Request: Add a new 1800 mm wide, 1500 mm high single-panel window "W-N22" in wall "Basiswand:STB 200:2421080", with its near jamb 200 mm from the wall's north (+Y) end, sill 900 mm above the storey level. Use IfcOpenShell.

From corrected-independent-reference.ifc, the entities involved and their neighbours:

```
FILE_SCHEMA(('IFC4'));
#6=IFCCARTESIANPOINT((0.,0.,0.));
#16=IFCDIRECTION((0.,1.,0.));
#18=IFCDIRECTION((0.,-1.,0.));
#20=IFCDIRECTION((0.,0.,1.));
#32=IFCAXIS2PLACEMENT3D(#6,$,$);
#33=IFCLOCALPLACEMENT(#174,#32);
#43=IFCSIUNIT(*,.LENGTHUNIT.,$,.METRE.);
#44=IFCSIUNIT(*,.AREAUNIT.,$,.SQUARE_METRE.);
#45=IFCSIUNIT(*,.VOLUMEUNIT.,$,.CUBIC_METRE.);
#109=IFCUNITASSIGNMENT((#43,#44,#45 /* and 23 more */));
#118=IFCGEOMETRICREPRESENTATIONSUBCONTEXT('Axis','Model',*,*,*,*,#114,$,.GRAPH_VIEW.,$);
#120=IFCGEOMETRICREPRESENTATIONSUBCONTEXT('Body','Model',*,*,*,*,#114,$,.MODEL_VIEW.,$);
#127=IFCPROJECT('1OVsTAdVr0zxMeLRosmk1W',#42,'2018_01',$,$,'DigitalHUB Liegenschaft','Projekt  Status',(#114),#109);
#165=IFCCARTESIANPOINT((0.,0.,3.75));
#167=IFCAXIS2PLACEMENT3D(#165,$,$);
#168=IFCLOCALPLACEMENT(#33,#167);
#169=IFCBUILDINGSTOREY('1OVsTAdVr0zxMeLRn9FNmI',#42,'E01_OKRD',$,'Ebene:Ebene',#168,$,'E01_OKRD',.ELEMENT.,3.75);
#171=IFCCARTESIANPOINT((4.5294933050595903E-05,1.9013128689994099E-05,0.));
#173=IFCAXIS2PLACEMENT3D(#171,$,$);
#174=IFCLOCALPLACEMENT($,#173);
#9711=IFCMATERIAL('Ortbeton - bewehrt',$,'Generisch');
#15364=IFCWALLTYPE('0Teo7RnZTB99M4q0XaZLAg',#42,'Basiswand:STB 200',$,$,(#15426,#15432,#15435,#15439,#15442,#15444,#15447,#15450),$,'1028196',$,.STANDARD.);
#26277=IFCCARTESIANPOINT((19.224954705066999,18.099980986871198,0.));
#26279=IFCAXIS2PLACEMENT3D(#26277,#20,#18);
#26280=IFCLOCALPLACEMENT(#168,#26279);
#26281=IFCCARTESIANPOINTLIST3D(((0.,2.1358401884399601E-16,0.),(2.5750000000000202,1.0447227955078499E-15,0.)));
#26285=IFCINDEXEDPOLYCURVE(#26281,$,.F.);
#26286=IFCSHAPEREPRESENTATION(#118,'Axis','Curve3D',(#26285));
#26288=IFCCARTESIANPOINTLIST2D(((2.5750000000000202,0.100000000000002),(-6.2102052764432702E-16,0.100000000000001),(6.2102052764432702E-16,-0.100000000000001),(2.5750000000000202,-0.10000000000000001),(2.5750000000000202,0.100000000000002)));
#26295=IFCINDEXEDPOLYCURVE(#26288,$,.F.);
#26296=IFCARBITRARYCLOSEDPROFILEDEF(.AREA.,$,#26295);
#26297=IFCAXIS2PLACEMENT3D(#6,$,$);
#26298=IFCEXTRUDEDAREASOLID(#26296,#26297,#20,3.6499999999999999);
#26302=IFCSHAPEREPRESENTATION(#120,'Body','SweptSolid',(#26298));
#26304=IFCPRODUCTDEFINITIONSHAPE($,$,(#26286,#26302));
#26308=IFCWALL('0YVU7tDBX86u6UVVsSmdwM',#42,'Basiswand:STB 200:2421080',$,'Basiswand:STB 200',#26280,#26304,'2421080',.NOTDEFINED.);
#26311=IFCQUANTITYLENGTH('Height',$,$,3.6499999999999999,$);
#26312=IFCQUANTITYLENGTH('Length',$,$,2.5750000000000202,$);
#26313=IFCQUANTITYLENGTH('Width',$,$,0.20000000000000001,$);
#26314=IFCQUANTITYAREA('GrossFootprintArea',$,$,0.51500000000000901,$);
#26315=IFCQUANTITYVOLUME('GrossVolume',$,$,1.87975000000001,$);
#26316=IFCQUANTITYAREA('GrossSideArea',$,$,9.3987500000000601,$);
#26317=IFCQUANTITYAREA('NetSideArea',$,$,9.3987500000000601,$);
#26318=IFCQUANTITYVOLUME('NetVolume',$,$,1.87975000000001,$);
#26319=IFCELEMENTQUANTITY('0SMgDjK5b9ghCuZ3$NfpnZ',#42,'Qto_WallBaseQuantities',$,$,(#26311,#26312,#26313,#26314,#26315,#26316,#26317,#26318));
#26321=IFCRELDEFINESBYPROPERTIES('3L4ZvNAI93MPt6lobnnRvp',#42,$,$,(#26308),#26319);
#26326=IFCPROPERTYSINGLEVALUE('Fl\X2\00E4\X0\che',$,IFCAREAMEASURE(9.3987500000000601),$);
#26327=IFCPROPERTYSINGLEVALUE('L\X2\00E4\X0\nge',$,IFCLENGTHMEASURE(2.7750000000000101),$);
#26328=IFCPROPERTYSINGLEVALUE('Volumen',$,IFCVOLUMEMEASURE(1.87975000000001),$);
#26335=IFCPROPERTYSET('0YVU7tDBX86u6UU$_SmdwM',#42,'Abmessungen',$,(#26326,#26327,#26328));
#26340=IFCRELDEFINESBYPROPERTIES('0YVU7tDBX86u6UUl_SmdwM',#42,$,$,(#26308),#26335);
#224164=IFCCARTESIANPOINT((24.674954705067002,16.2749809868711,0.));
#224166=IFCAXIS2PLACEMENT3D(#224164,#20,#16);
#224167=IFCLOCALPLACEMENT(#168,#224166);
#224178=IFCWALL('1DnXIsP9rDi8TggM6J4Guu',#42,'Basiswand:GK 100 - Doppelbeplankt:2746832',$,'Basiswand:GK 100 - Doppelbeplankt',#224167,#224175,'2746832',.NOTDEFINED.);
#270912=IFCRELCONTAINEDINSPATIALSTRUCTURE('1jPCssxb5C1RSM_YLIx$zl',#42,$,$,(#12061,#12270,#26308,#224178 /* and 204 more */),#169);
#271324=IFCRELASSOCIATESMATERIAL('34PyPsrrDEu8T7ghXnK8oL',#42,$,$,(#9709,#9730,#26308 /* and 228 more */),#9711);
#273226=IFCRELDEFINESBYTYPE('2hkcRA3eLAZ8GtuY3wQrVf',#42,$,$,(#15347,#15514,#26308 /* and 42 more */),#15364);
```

```python
import numpy as np
import ifcopenshell
import ifcopenshell.api.feature
import ifcopenshell.api.geometry
import ifcopenshell.api.pset
import ifcopenshell.api.root
import ifcopenshell.api.spatial
import ifcopenshell.geom
import ifcopenshell.util.element
import ifcopenshell.util.placement
import ifcopenshell.util.representation
import ifcopenshell.util.shape
import ifcopenshell.util.unit

model = ifcopenshell.open("corrected-independent-reference.ifc")
unit_scale = ifcopenshell.util.unit.calculate_unit_scale(model)
area_scale = ifcopenshell.util.unit.calculate_unit_scale(model, "AREAUNIT")
volume_scale = ifcopenshell.util.unit.calculate_unit_scale(model, "VOLUMEUNIT")
settings = ifcopenshell.geom.settings()


def volume(element):
    """Net volume in cubic metres, openings subtracted."""
    shape = ifcopenshell.geom.create_shape(settings, element)
    return ifcopenshell.util.shape.get_volume(shape.geometry)


wall = model.by_guid("0YVU7tDBX86u6UVVsSmdwM")
storey = ifcopenshell.util.element.get_container(wall, ifc_class="IfcBuildingStorey")
context = ifcopenshell.util.representation.get_context(model, "Model", "Body", "MODEL_VIEW")
before = volume(wall)

width, height, from_end, sill = 1.8, 1.5, 0.2, 0.9  # metres

# The wall runs along its own X axis, and the end named is its -X end.
wall_shape = ifcopenshell.geom.create_shape(settings, wall)
x, y, z = ifcopenshell.util.shape.get_vertices(wall_shape.geometry).T
start = x.min() + from_end
face, thickness = float(y.min()), float(y.max() - y.min())
wall_matrix = ifcopenshell.util.placement.get_local_placement(wall.ObjectPlacement)
level = ifcopenshell.util.placement.get_local_placement(storey.ObjectPlacement)[2, 3]


def in_wall(x, y):
    """Placement at x, y metres in the wall's axes, at sill height."""
    matrix = wall_matrix.copy()
    matrix[:, 3] = wall_matrix @ np.array([x / unit_scale, y / unit_scale, 0.0, 1.0])
    matrix[2, 3] = level + sill / unit_scale
    return matrix


# Opening: a box that overshoots both wall faces by 50 mm.
opening = ifcopenshell.api.root.create_entity(model, ifc_class="IfcOpeningElement", predefined_type="OPENING")
box = ifcopenshell.api.geometry.add_wall_representation(
    model, context=context, length=width, height=height, thickness=thickness + 0.1
)
ifcopenshell.api.geometry.assign_representation(model, product=opening, representation=box)
ifcopenshell.api.geometry.edit_object_placement(model, product=opening, matrix=in_wall(start, face - 0.05), is_si=False)
ifcopenshell.api.feature.add_feature(model, feature=opening, element=wall)

window = ifcopenshell.api.root.create_entity(model, ifc_class="IfcWindow", name="W-N22", predefined_type="WINDOW")
window.OverallWidth, window.OverallHeight = width / unit_scale, height / unit_scale
window.PartitioningType = "SINGLE_PANEL"
body = ifcopenshell.api.geometry.add_window_representation(
    model,
    context=context,
    overall_width=window.OverallWidth,
    overall_height=window.OverallHeight,
    partition_type="SINGLE_PANEL",
)
ifcopenshell.api.geometry.assign_representation(model, product=window, representation=body)
ifcopenshell.api.spatial.assign_container(model, products=[window], relating_structure=storey)
ifcopenshell.api.feature.add_filling(model, opening=opening, element=window)

# Centre the window in the wall's thickness.
ifcopenshell.api.geometry.edit_object_placement(model, product=window, matrix=in_wall(start, face), is_si=False)
window_shape = ifcopenshell.geom.create_shape(settings, window)
depth = ifcopenshell.util.shape.get_vertices(window_shape.geometry)[:, 1]
offset = face + thickness / 2 - (depth.min() + depth.max()) / 2
ifcopenshell.api.geometry.edit_object_placement(model, product=window, matrix=in_wall(start, offset), is_si=False)

after = volume(wall)

# Update the wall's stored quantities.
qto = model.by_id(ifcopenshell.util.element.get_pset(wall, "Qto_WallBaseQuantities", should_inherit=False)["id"])
ifcopenshell.api.pset.edit_qto(model, qto=qto, properties={
    "NetSideArea": after / thickness / area_scale,
    "NetVolume": after / volume_scale,
})
pset = model.by_id(ifcopenshell.util.element.get_pset(wall, "Abmessungen", should_inherit=False)["id"])
ifcopenshell.api.pset.edit_pset(model, pset=pset, properties={
    "Fläche": model.create_entity("IfcAreaMeasure", after / thickness / area_scale),
    "Volumen": model.create_entity("IfcVolumeMeasure", after / volume_scale),
})

print(f"wall volume {before:.3f} -> {after:.3f} m3")

model.write("corrected-independent-reference-out.ifc")
```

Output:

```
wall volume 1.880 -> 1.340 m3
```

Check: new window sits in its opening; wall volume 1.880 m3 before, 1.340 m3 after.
